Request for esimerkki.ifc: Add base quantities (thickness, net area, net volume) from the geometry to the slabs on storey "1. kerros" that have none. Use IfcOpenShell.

First a look at what the model holds.

```python
import ifcopenshell
import ifcopenshell.util.element
import ifcopenshell.util.unit

model = ifcopenshell.open("esimerkki.ifc")
print(model.schema)
for unit_type in ("LENGTHUNIT", "AREAUNIT", "VOLUMEUNIT"):
    print(unit_type, ifcopenshell.util.unit.calculate_unit_scale(model, unit_type))
storey = next(s for s in model.by_type("IfcBuildingStorey") if s.Name == "1. kerros")
slabs = [e for e in ifcopenshell.util.element.get_decomposition(storey) if e.is_a("IfcSlab")]
for e in sorted(slabs, key=lambda e: e.id()):
    print(e.id(), e.is_a(), e.Name, list(ifcopenshell.util.element.get_psets(e, qtos_only=True)), sep=" | ")
```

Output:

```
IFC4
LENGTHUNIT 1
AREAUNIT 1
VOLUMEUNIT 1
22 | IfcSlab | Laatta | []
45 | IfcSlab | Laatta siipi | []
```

```python
import ifcopenshell
import ifcopenshell.api.pset
import ifcopenshell.geom
import ifcopenshell.util.element
import ifcopenshell.util.shape
import ifcopenshell.util.unit

model = ifcopenshell.open("esimerkki.ifc")
unit_scale = ifcopenshell.util.unit.calculate_unit_scale(model)
area_scale = ifcopenshell.util.unit.calculate_unit_scale(model, "AREAUNIT")
volume_scale = ifcopenshell.util.unit.calculate_unit_scale(model, "VOLUMEUNIT")
settings = ifcopenshell.geom.settings()

storey = next(s for s in model.by_type("IfcBuildingStorey") if s.Name == "1. kerros")
slabs = [e for e in ifcopenshell.util.element.get_decomposition(storey) if e.is_a("IfcSlab")]

for e in sorted(slabs, key=lambda e: e.id()):
    if ifcopenshell.util.element.get_psets(e, qtos_only=True, should_inherit=False):
        continue
    # Geometry comes back in metres, in the element's own axes.
    shape = ifcopenshell.geom.create_shape(settings, e)
    values = {
        "Width": ifcopenshell.util.shape.get_z(shape.geometry) / unit_scale,
        "NetArea": ifcopenshell.util.shape.get_footprint_area(shape.geometry) / area_scale,
        "NetVolume": ifcopenshell.util.shape.get_volume(shape.geometry) / volume_scale,
    }
    qto = ifcopenshell.api.pset.add_qto(model, product=e, name="Qto_SlabBaseQuantities")
    ifcopenshell.api.pset.edit_qto(model, qto=qto, properties=values)
    print(e.id(), {k: round(v, 3) for k, v in values.items()})

model.write("esimerkki-out.ifc")
```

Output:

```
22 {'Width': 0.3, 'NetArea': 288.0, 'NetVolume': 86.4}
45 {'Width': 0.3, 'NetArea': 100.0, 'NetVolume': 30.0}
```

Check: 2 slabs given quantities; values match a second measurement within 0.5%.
